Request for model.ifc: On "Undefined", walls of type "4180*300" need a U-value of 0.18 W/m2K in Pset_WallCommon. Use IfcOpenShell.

First a look at what the model holds.

```python
import ifcopenshell
import ifcopenshell.util.element

model = ifcopenshell.open("model.ifc")
print(model.schema)
storey = next(s for s in model.by_type("IfcBuildingStorey") if s.Name == "Undefined")
walls = [e for e in ifcopenshell.util.element.get_decomposition(storey) if e.is_a("IfcWall")]
seen = {}
for e in walls:
    element_type = ifcopenshell.util.element.get_type(e)
    key = (element_type.Name if element_type != e and element_type else None, ifcopenshell.util.element.get_pset(e, "Pset_WallCommon", "ThermalTransmittance"))
    seen[key] = seen.get(key, 0) + 1
for (name, value), count in sorted(seen.items(), key=str):
    print(count, "x", name, "|", value)
```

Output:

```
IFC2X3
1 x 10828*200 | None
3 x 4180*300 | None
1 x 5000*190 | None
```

```python
import ifcopenshell
import ifcopenshell.api.pset
import ifcopenshell.util.element

model = ifcopenshell.open("model.ifc")

storey = next(s for s in model.by_type("IfcBuildingStorey") if s.Name == "Undefined")
walls = [e for e in ifcopenshell.util.element.get_decomposition(storey) if e.is_a("IfcWall")]

count = 0
for e in walls:
    element_type = ifcopenshell.util.element.get_type(e)
    if element_type in (None, e) or element_type.Name != "4180*300":
        continue
    found = ifcopenshell.util.element.get_pset(e, "Pset_WallCommon", should_inherit=False)
    if found:
        pset = model.by_id(found["id"])
        if len(ifcopenshell.util.element.get_elements_by_pset(pset)) > 1:
            pset = ifcopenshell.api.pset.unshare_pset(model, products=[e], pset=pset)[0]
    else:
        pset = ifcopenshell.api.pset.add_pset(model, product=e, name="Pset_WallCommon")
    ifcopenshell.api.pset.edit_pset(model, pset=pset, properties={"ThermalTransmittance": 0.18})
    count += 1

print(count, "walls updated")

model.write("model_edited.ifc")
```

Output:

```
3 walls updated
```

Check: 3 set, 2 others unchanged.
